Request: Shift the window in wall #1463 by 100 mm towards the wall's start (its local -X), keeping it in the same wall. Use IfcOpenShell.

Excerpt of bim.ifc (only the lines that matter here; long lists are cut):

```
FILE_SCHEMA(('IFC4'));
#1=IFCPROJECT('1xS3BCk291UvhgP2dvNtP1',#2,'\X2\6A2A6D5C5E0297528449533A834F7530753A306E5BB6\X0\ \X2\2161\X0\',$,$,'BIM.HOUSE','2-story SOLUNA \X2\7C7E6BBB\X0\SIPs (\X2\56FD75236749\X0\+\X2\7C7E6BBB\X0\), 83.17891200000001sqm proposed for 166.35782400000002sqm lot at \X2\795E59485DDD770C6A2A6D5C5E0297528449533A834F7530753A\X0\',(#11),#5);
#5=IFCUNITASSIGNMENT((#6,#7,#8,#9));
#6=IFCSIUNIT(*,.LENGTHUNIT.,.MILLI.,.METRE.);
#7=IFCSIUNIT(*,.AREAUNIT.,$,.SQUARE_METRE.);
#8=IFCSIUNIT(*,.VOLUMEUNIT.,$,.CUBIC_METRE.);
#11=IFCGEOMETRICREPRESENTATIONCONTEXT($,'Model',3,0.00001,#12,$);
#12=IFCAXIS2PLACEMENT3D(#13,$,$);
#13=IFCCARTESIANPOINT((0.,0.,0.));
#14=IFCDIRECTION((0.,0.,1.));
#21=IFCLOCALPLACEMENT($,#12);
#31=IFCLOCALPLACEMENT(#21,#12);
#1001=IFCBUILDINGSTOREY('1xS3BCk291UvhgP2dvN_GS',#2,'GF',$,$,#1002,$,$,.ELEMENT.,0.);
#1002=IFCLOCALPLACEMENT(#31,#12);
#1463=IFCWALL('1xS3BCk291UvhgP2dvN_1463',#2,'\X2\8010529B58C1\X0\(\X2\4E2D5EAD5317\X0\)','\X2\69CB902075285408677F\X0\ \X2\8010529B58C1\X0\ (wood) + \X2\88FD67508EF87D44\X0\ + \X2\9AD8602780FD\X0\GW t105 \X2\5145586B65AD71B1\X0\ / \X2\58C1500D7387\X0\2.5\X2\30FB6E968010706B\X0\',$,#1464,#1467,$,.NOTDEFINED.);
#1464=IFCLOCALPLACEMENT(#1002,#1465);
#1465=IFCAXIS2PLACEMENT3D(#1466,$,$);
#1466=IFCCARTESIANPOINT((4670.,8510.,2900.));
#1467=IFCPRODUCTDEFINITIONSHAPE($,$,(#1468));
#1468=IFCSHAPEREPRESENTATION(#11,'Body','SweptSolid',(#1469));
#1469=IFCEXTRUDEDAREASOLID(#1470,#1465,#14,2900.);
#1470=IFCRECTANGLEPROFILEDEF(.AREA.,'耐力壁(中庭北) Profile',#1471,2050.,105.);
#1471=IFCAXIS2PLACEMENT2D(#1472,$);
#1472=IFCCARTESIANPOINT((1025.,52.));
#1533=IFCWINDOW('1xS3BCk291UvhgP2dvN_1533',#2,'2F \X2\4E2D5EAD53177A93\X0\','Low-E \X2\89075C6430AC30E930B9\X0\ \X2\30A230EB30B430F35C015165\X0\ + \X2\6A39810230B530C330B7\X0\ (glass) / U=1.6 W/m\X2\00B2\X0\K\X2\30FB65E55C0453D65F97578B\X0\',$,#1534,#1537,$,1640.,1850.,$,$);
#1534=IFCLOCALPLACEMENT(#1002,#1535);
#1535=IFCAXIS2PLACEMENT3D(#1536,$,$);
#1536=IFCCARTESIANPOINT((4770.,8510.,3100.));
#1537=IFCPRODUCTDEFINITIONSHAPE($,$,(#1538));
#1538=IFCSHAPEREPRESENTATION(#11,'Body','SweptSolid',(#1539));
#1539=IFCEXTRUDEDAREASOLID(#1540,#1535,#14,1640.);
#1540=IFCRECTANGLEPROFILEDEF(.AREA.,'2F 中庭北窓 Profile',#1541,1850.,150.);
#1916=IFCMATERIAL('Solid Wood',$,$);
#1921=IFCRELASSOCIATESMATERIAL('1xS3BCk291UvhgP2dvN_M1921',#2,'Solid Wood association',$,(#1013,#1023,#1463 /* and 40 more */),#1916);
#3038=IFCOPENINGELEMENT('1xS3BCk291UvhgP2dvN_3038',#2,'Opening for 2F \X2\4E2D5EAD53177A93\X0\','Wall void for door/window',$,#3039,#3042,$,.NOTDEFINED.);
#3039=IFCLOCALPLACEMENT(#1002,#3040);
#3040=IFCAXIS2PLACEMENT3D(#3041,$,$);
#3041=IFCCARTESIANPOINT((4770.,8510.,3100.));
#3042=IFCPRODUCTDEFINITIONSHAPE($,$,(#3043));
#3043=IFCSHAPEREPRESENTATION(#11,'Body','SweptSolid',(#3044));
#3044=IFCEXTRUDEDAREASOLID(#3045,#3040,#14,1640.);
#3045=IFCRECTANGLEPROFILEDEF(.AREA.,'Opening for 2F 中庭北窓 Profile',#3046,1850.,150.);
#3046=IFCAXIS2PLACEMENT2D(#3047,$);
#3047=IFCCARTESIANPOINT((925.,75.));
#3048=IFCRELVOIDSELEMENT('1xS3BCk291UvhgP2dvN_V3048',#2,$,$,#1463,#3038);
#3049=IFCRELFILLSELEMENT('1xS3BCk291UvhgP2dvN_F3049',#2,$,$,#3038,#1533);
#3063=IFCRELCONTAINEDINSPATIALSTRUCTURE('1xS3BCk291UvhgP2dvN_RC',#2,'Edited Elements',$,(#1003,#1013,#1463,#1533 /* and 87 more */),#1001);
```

```python
import ifcopenshell
import ifcopenshell.api.geometry
import ifcopenshell.util.placement
import ifcopenshell.util.unit

model = ifcopenshell.open("bim.ifc")
unit_scale = ifcopenshell.util.unit.calculate_unit_scale(model)

window = model.by_guid("1xS3BCk291UvhgP2dvN_1533")
opening = window.FillsVoids[0].RelatingOpeningElement
wall = opening.VoidsElements[0].RelatingBuildingElement

wall_matrix = ifcopenshell.util.placement.get_local_placement(wall.ObjectPlacement)
shift = wall_matrix[:3, 0] * -0.1 / unit_scale
before = ifcopenshell.util.placement.get_local_placement(window.ObjectPlacement)[:3, 3].copy()

# The window is not placed relative to its opening, so move both.
for product in (opening, window):
    matrix = ifcopenshell.util.placement.get_local_placement(product.ObjectPlacement)
    matrix[:3, 3] += shift
    ifcopenshell.api.geometry.edit_object_placement(model, product=product, matrix=matrix, is_si=False)

after = ifcopenshell.util.placement.get_local_placement(window.ObjectPlacement)[:3, 3]
print("window moved by", (after - before).round(3) + 0.0)

model.write("bim_updated.ifc")
```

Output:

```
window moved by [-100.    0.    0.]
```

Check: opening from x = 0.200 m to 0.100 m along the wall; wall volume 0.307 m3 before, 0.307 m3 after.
